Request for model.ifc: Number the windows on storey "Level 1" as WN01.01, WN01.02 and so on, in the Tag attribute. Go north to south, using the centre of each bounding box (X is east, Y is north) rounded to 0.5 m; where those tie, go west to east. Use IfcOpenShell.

First a look at what the model holds.

```python
import ifcopenshell
import ifcopenshell.util.element
import ifcopenshell.util.placement

model = ifcopenshell.open("model.ifc")
print(model.schema)
storey = next(s for s in model.by_type("IfcBuildingStorey") if s.Name == "Level 1")
windows = [e for e in ifcopenshell.util.element.get_decomposition(storey) if e.is_a("IfcWindow")]
for e in sorted(windows, key=lambda e: e.id()):
    origin = ifcopenshell.util.placement.get_local_placement(e.ObjectPlacement)[:3, 3]
    print(e.id(), e.Tag, e.Name, origin.round(2) + 0.0, sep=" | ")
```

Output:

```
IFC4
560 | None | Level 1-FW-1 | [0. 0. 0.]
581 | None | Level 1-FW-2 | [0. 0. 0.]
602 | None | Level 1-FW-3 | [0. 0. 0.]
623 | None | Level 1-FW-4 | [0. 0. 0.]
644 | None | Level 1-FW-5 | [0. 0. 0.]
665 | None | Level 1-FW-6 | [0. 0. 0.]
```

```python
import ifcopenshell
import ifcopenshell.geom
import ifcopenshell.util.element
import ifcopenshell.util.shape

model = ifcopenshell.open("model.ifc")
settings = ifcopenshell.geom.settings()
settings.set("use-world-coords", True)


def centre(element):
    shape = ifcopenshell.geom.create_shape(settings, element)
    return ifcopenshell.util.shape.get_bbox_centroid(shape.geometry)


storey = next(s for s in model.by_type("IfcBuildingStorey") if s.Name == "Level 1")
windows = [e for e in ifcopenshell.util.element.get_decomposition(storey) if e.is_a("IfcWindow")]

# Insertion points can sit at a corner or the storey origin, so sort by the geometry (in metres).
centres = {e: centre(e) for e in windows}
windows.sort(key=lambda e: (-round(centres[e][1] / 0.5), centres[e][0]))

for i, e in enumerate(windows, start=1):
    number = f"WN01.{i:02d}"
    e.Tag = number
    print(e.id(), number)

model.write("model_rev.ifc")
```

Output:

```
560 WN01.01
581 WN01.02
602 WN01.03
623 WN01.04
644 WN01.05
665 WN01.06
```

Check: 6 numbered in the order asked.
